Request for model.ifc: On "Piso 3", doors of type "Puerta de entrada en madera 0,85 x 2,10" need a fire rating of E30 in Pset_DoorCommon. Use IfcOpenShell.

First a look at what the model holds.

```python
import ifcopenshell
import ifcopenshell.util.element

model = ifcopenshell.open("model.ifc")
print(model.schema)
storey = next(s for s in model.by_type("IfcBuildingStorey") if s.Name == "Piso 3")
doors = [e for e in ifcopenshell.util.element.get_decomposition(storey) if e.is_a("IfcDoor")]
seen = {}
for e in doors:
    element_type = ifcopenshell.util.element.get_type(e)
    key = (element_type.Name if element_type != e and element_type else None, ifcopenshell.util.element.get_pset(e, "Pset_DoorCommon", "FireRating"))
    seen[key] = seen.get(key, 0) + 1
for (name, value), count in sorted(seen.items(), key=str):
    print(count, "x", name, "|", value)
```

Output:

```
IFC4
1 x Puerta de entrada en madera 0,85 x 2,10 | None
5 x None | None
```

```python
import ifcopenshell
import ifcopenshell.api.pset
import ifcopenshell.util.element

model = ifcopenshell.open("model.ifc")

storey = next(s for s in model.by_type("IfcBuildingStorey") if s.Name == "Piso 3")
doors = [e for e in ifcopenshell.util.element.get_decomposition(storey) if e.is_a("IfcDoor")]

count = 0
for e in doors:
    element_type = ifcopenshell.util.element.get_type(e)
    if element_type in (None, e) or element_type.Name != "Puerta de entrada en madera 0,85 x 2,10":
        continue
    # add_pset returns the element's existing set when there is one.
    pset = ifcopenshell.api.pset.add_pset(model, product=e, name="Pset_DoorCommon")
    ifcopenshell.api.pset.edit_pset(model, pset=pset, properties={"FireRating": "E30"})
    count += 1

print(count, "doors updated")

model.write("model_rev.ifc")
```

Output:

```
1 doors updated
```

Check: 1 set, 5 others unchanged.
